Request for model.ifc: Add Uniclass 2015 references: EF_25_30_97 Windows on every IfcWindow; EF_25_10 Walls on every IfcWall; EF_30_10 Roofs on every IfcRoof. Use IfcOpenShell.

First a look at what the model holds.

```python
import ifcopenshell

model = ifcopenshell.open("model.ifc")
print(model.schema)
print("classifications:", [c.Name for c in model.by_type("IfcClassification")])
for ifc_class in ("IfcDoor", "IfcRoof", "IfcStair", "IfcWall", "IfcWindow"):
    print(ifc_class, len(model.by_type(ifc_class)))
```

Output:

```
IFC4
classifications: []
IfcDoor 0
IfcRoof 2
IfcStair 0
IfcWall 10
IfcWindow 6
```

```python
import ifcopenshell
import ifcopenshell.api.classification

model = ifcopenshell.open("model.ifc")

system = ifcopenshell.api.classification.add_classification(model, classification="Uniclass 2015")

codes = {
    "IfcWindow": ("EF_25_30_97", "Windows"),
    "IfcWall": ("EF_25_10", "Walls"),
    "IfcRoof": ("EF_30_10", "Roofs"),
}
for ifc_class, (code, name) in codes.items():
    products = model.by_type(ifc_class)
    ifcopenshell.api.classification.add_reference(
        model, products=products, classification=system, identification=code, name=name
    )
    print(code, len(products))

model.write("model_updated.ifc")
```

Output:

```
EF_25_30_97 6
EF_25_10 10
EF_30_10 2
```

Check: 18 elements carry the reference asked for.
